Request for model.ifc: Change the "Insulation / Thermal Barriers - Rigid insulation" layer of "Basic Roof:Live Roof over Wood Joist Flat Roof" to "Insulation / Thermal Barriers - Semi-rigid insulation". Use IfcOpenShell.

First a look at what the model holds.

```python
import ifcopenshell
import ifcopenshell.util.element

model = ifcopenshell.open("model.ifc")
print(model.schema)
for layer_set in model.by_type("IfcMaterialLayerSet"):
    if layer_set.LayerSetName == "Basic Roof:Live Roof over Wood Joist Flat Roof":
        for layer in layer_set.MaterialLayers:
            print(layer.id(), layer.Material and layer.Material.Name, layer.LayerThickness, sep=" | ")
        print(len(ifcopenshell.util.element.get_elements_by_material(model, layer_set)), "elements and types use it")
print(sorted(m.Name for m in model.by_type("IfcMaterial") if m.Name)[:60])
```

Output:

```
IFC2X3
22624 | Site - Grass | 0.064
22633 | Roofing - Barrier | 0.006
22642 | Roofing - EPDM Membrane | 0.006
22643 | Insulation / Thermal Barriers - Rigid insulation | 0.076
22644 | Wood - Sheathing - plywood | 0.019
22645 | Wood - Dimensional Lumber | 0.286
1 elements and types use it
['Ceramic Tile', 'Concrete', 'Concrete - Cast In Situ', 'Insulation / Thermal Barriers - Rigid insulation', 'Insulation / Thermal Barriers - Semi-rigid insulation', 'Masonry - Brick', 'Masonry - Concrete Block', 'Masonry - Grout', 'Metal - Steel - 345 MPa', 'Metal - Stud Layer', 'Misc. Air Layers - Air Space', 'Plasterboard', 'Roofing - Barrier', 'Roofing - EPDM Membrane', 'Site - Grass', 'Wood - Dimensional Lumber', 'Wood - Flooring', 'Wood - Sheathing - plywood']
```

```python
import ifcopenshell
import ifcopenshell.api.material

model = ifcopenshell.open("model.ifc")

layer_set = next(s for s in model.by_type("IfcMaterialLayerSet") if s.LayerSetName == "Basic Roof:Live Roof over Wood Joist Flat Roof")
layer = next(l for l in layer_set.MaterialLayers if l.Material and l.Material.Name == "Insulation / Thermal Barriers - Rigid insulation")
material = next(m for m in model.by_type("IfcMaterial") if m.Name == "Insulation / Thermal Barriers - Semi-rigid insulation")

# Point this one layer at the other material; renaming the old one would change it everywhere.
ifcopenshell.api.material.edit_layer(model, layer=layer, attributes={}, material=material)

print([l.Material.Name if l.Material else None for l in layer_set.MaterialLayers])

model.write("model_v2.ifc")
```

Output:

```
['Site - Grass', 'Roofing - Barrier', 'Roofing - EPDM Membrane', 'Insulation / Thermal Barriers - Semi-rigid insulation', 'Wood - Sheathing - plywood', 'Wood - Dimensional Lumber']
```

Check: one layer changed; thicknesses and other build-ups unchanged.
